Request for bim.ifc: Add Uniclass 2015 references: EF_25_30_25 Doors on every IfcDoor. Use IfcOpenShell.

First a look at what the model holds.

```python
import ifcopenshell

model = ifcopenshell.open("bim.ifc")
print(model.schema)
print("classifications:", [c.Name for c in model.by_type("IfcClassification")])
for ifc_class in ("IfcDoor", "IfcRoof", "IfcStair", "IfcWall", "IfcWindow"):
    print(ifc_class, len(model.by_type(ifc_class)))
```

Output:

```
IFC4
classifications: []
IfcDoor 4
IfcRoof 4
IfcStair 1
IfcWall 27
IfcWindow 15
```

```python
import ifcopenshell
import ifcopenshell.api.classification

model = ifcopenshell.open("bim.ifc")

system = ifcopenshell.api.classification.add_classification(model, classification="Uniclass 2015")

codes = {
    "IfcDoor": ("EF_25_30_25", "Doors"),
}
for ifc_class, (code, name) in codes.items():
    products = model.by_type(ifc_class)
    ifcopenshell.api.classification.add_reference(
        model, products=products, classification=system, identification=code, name=name
    )
    print(code, len(products))

model.write("bim_v2.ifc")
```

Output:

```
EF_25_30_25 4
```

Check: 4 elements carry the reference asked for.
